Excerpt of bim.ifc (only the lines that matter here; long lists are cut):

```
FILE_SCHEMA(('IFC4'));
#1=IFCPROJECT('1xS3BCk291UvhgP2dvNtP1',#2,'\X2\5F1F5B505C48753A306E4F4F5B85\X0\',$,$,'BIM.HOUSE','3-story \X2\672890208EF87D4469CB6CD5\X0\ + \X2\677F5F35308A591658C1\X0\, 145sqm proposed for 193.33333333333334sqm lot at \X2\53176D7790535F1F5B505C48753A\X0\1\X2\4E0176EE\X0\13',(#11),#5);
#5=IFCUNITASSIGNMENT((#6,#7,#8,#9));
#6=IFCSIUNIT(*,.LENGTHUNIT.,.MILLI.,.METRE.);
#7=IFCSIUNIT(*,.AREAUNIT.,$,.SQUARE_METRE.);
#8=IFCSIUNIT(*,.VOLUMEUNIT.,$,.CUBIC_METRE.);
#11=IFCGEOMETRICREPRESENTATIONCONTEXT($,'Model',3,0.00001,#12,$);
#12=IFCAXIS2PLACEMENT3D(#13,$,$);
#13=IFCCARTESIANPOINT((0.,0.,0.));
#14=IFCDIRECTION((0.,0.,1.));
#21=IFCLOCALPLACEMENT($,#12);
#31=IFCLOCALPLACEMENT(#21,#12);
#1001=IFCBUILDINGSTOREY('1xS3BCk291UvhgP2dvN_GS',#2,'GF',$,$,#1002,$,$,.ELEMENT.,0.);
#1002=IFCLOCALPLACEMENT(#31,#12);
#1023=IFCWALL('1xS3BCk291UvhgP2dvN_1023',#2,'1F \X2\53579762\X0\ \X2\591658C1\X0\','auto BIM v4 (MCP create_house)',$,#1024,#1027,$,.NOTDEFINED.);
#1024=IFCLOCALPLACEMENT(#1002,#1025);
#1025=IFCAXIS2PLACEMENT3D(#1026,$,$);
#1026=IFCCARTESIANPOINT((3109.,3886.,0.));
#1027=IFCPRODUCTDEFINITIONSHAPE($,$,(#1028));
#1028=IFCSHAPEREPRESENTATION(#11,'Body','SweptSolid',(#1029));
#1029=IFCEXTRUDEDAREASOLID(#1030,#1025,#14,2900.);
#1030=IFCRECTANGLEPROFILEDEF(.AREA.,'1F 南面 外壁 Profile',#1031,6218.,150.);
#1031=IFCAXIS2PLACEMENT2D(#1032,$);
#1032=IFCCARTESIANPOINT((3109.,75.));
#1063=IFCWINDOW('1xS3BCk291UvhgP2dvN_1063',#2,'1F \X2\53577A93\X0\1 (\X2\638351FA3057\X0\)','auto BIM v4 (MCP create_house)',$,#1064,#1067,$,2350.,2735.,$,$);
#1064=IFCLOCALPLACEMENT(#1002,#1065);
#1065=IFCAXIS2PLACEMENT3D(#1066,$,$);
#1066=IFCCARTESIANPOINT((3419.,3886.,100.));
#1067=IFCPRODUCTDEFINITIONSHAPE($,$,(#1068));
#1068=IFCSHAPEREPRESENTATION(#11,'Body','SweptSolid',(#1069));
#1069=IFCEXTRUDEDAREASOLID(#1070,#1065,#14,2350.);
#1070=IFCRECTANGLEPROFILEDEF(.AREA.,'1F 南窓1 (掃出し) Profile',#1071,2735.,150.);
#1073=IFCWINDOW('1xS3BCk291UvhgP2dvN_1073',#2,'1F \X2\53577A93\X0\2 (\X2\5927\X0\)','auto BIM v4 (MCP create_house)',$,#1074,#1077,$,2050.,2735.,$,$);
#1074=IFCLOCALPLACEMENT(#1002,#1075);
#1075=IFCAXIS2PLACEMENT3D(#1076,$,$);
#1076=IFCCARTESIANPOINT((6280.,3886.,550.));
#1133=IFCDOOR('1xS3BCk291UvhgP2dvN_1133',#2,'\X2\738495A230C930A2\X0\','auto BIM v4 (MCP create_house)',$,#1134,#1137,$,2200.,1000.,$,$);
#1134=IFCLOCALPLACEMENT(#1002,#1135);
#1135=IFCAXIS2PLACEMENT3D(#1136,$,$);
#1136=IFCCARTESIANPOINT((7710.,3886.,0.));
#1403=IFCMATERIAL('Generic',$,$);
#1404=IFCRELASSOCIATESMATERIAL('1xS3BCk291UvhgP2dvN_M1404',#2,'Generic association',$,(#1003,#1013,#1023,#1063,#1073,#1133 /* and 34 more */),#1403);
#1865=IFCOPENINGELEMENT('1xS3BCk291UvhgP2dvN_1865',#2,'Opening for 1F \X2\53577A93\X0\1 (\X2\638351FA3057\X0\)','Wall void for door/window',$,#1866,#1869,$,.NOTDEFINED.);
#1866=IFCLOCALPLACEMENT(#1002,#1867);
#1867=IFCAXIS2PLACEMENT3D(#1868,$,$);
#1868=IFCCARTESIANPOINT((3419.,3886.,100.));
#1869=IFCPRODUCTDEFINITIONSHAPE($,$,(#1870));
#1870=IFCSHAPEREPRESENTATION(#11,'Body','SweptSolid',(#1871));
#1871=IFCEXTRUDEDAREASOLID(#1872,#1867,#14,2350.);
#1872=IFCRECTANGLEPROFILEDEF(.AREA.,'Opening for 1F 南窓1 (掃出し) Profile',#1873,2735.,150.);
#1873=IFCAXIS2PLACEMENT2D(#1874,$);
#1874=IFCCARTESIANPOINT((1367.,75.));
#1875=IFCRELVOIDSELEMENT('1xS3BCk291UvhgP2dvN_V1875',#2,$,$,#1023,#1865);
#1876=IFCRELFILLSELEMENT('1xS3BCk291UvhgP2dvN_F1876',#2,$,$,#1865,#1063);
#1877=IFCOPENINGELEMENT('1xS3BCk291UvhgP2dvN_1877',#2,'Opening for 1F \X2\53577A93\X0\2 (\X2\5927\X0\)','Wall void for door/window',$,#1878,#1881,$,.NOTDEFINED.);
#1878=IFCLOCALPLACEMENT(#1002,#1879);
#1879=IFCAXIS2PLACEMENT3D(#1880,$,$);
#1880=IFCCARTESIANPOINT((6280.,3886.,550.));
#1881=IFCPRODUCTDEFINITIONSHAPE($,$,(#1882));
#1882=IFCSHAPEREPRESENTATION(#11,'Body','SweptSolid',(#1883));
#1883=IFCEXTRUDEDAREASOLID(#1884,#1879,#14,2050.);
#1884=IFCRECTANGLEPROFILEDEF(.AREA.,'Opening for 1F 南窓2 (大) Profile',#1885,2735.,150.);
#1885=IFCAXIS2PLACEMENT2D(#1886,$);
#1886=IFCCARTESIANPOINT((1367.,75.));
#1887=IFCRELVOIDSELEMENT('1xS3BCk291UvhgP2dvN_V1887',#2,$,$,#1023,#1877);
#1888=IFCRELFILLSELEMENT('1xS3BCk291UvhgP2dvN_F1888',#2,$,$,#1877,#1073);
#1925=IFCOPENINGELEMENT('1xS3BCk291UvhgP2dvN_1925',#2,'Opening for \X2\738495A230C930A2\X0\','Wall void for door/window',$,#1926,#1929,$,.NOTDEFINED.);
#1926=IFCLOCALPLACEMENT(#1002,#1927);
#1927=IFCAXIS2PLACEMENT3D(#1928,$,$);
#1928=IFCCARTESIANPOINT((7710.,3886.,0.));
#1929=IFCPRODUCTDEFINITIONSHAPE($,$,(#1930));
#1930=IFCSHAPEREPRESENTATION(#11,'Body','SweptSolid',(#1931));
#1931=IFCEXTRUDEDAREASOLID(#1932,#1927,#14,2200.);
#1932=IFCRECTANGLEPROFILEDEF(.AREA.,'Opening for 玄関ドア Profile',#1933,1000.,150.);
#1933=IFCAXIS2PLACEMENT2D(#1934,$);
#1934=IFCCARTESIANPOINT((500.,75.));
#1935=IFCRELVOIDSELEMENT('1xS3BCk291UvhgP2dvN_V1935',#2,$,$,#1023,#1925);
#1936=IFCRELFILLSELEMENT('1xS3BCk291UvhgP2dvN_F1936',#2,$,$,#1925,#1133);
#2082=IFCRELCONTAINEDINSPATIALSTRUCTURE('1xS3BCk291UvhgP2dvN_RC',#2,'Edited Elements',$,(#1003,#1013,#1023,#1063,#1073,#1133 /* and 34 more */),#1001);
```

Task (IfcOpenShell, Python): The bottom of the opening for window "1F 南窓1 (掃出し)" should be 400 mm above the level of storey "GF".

```python
import numpy as np
import ifcopenshell
import ifcopenshell.api.geometry
import ifcopenshell.geom
import ifcopenshell.util.element
import ifcopenshell.util.placement
import ifcopenshell.util.shape
import ifcopenshell.util.unit

model = ifcopenshell.open("bim.ifc")
unit_scale = ifcopenshell.util.unit.calculate_unit_scale(model)

window = model.by_guid("1xS3BCk291UvhgP2dvN_1063")
opening = window.FillsVoids[0].RelatingOpeningElement
storey = ifcopenshell.util.element.get_container(window, ifc_class="IfcBuildingStorey")
level = ifcopenshell.util.placement.get_local_placement(storey.ObjectPlacement)[2, 3]

# The opening's origin need not be at the sill, so measure its lowest point.
shape = ifcopenshell.geom.create_shape(ifcopenshell.geom.settings(), opening)
bottom = ifcopenshell.util.shape.get_shape_bottom_elevation(shape, shape.geometry) / unit_scale
dz = level + 400.0 - bottom

shift = np.array([0.0, 0.0, dz])
# The window is not placed relative to its opening, so move both.
for product in (opening, window):
    matrix = ifcopenshell.util.placement.get_local_placement(product.ObjectPlacement)
    matrix[:3, 3] += shift
    ifcopenshell.api.geometry.edit_object_placement(model, product=product, matrix=matrix, is_si=False)

print(f"moved by {dz * unit_scale:+.3f} m")

model.write("bim_edited.ifc")
```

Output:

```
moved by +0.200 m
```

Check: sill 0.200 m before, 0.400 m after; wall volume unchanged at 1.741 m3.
